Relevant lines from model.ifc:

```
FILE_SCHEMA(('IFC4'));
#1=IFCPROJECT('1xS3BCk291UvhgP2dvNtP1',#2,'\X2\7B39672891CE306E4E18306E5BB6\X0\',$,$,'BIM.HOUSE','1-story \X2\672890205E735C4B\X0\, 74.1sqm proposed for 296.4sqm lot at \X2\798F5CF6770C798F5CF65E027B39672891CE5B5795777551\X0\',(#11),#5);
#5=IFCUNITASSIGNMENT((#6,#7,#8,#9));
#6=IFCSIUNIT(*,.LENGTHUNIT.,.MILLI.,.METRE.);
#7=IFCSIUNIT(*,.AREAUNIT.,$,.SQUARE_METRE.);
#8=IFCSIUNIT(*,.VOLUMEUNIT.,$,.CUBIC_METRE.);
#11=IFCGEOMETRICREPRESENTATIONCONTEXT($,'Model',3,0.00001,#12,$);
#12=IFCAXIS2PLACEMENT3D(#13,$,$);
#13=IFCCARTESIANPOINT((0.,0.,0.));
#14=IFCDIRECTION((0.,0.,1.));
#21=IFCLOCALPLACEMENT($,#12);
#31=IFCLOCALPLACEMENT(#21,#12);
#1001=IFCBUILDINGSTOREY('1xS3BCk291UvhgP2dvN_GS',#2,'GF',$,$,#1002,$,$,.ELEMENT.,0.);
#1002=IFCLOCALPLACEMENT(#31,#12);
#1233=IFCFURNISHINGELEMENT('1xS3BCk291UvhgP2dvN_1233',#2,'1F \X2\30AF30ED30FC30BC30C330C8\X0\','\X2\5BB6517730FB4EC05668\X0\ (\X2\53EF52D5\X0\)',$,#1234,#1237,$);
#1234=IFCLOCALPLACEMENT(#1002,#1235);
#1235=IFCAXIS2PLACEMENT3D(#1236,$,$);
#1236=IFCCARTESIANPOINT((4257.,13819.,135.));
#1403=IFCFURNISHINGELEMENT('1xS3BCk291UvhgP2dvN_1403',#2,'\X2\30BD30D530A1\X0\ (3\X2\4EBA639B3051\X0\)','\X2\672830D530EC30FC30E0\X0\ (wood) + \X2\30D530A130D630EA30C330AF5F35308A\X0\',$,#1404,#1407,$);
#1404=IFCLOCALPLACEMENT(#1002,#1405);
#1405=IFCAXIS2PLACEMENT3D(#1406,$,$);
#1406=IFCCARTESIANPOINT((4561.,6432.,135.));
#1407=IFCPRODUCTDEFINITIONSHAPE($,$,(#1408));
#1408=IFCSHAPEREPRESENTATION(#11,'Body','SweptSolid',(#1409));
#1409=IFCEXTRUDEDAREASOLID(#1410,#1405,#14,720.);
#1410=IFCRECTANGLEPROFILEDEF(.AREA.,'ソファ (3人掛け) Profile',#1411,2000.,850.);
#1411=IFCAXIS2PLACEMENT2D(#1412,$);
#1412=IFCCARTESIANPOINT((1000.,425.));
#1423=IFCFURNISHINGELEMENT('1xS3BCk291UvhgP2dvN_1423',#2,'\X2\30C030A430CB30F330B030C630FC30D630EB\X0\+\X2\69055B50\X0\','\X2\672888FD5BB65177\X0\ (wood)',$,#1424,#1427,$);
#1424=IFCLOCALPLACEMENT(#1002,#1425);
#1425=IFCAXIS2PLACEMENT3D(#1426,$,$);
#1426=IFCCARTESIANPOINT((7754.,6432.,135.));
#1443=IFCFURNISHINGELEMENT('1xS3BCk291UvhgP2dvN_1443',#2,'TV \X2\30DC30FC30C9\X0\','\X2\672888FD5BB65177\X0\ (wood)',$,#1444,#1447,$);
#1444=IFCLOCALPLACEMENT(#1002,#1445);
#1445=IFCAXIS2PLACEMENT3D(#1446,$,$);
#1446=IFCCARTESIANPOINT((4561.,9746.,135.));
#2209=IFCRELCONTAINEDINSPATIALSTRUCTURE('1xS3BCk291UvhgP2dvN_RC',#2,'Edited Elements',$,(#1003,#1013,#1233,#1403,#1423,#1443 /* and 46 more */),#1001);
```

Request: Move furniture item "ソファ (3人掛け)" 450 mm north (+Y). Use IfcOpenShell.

```python
import ifcopenshell
import ifcopenshell.api.geometry
import ifcopenshell.util.placement
import ifcopenshell.util.unit

model = ifcopenshell.open("model.ifc")
unit_scale = ifcopenshell.util.unit.calculate_unit_scale(model)

item = model.by_guid("1xS3BCk291UvhgP2dvN_1403")
matrix = ifcopenshell.util.placement.get_local_placement(item.ObjectPlacement)
matrix[1, 3] += 0.45 / unit_scale
ifcopenshell.api.geometry.edit_object_placement(model, product=item, matrix=matrix, is_si=False)

print(ifcopenshell.util.placement.get_local_placement(item.ObjectPlacement).round(3) + 0.0)

model.write("model_rev.ifc")
```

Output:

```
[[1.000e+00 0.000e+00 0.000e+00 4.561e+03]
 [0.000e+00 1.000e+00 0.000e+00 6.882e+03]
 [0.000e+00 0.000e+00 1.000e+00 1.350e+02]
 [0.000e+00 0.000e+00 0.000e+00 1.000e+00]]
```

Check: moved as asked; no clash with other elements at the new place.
